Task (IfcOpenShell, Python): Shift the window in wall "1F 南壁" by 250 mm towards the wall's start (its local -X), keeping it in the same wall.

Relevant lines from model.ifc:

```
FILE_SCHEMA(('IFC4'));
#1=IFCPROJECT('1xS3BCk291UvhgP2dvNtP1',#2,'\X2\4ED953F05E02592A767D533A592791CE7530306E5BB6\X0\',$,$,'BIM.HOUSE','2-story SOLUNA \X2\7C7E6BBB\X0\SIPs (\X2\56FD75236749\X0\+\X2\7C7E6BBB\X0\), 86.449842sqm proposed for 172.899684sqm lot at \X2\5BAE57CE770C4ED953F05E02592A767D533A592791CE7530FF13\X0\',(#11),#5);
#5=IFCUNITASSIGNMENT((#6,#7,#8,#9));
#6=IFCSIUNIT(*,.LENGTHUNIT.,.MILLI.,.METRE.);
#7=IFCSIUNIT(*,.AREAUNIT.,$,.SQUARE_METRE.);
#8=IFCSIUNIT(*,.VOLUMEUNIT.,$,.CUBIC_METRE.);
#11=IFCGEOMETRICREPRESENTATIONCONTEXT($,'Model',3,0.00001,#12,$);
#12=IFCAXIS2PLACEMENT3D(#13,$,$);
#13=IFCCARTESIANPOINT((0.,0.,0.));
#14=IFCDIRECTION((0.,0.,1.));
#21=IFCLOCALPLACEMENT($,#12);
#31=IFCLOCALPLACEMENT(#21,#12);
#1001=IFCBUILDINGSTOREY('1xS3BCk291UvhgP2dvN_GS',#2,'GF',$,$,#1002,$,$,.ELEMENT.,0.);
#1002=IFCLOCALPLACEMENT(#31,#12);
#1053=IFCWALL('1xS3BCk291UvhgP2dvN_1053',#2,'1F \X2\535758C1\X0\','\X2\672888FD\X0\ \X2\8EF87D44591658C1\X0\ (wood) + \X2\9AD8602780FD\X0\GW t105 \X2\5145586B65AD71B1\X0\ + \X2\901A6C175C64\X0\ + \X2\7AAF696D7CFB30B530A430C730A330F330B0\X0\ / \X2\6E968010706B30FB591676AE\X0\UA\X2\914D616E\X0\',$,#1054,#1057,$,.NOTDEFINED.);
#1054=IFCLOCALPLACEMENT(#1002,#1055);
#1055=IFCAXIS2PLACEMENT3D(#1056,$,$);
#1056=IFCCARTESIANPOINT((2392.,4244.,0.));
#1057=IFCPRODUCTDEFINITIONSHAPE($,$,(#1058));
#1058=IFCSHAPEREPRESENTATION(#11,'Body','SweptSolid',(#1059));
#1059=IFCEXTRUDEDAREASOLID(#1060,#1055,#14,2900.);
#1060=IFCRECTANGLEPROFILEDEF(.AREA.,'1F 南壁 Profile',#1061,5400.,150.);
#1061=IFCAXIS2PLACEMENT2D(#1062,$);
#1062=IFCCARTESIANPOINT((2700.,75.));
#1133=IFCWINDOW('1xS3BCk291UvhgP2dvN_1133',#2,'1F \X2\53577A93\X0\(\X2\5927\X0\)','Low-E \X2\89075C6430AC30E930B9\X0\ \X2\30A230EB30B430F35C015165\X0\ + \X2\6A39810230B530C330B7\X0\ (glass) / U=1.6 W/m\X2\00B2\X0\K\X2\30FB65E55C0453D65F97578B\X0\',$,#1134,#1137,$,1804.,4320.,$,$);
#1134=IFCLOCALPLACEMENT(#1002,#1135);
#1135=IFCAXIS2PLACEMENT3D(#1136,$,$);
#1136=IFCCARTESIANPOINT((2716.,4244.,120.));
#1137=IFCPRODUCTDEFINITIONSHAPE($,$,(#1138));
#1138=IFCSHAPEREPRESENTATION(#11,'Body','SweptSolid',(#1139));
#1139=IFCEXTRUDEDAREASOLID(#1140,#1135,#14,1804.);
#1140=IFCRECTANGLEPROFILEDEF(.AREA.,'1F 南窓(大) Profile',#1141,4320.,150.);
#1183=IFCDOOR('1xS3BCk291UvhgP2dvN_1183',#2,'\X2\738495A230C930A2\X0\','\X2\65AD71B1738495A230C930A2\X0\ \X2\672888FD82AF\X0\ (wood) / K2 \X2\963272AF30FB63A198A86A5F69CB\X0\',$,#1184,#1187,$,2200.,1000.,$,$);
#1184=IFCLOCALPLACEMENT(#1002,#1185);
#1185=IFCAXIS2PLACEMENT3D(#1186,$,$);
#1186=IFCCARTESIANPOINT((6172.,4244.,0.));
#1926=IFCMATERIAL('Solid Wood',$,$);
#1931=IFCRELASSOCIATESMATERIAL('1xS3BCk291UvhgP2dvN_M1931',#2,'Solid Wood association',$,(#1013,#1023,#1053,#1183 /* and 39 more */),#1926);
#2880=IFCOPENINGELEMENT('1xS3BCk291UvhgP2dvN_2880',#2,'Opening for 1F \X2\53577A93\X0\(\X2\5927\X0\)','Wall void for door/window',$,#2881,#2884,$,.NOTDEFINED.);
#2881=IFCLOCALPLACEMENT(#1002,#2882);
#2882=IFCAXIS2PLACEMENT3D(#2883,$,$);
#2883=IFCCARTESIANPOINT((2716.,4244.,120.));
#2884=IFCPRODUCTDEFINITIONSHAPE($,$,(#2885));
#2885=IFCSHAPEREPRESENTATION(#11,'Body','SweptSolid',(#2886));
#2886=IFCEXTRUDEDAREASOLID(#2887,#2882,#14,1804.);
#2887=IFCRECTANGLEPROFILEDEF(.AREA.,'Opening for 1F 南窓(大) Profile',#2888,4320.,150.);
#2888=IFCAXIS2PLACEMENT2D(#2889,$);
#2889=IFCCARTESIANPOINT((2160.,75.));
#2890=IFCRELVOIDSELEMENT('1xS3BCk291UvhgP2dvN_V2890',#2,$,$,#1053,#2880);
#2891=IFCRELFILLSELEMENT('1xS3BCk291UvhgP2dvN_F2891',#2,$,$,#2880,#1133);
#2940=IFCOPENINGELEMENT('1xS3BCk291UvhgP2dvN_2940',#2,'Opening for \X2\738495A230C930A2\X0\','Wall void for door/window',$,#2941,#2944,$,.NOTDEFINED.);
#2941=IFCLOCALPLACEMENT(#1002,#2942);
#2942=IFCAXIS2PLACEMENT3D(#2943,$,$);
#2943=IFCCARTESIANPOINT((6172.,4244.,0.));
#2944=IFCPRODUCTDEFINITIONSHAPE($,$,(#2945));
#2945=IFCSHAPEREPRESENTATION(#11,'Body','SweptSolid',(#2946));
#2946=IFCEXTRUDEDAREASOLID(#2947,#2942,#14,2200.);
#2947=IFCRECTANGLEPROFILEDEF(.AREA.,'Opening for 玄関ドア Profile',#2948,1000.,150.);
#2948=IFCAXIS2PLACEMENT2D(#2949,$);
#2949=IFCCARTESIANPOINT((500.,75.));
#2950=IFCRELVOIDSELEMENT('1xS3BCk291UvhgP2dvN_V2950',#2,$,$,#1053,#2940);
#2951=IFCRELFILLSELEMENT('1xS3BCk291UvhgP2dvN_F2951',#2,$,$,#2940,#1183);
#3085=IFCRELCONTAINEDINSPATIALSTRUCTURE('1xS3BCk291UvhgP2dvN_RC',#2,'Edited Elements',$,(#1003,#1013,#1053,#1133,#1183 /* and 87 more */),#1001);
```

```python
import ifcopenshell
import ifcopenshell.api.geometry
import ifcopenshell.util.placement
import ifcopenshell.util.unit

model = ifcopenshell.open("model.ifc")
unit_scale = ifcopenshell.util.unit.calculate_unit_scale(model)

window = model.by_guid("1xS3BCk291UvhgP2dvN_1133")
opening = window.FillsVoids[0].RelatingOpeningElement
wall = opening.VoidsElements[0].RelatingBuildingElement

wall_matrix = ifcopenshell.util.placement.get_local_placement(wall.ObjectPlacement)
shift = wall_matrix[:3, 0] * -0.25 / unit_scale
before = ifcopenshell.util.placement.get_local_placement(window.ObjectPlacement)[:3, 3].copy()

# The window is not placed relative to its opening, so move both.
for product in (opening, window):
    matrix = ifcopenshell.util.placement.get_local_placement(product.ObjectPlacement)
    matrix[:3, 3] += shift
    ifcopenshell.api.geometry.edit_object_placement(model, product=product, matrix=matrix, is_si=False)

after = ifcopenshell.util.placement.get_local_placement(window.ObjectPlacement)[:3, 3]
print("window moved by", (after - before).round(3) + 0.0)

model.write("model_updated.ifc")
```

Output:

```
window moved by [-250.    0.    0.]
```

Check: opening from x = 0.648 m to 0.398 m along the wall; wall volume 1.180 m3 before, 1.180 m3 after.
